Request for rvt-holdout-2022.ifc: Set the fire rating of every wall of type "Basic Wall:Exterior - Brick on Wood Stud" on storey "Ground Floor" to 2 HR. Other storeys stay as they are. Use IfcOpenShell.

First a look at what the model holds.

```python
import ifcopenshell
import ifcopenshell.util.element

model = ifcopenshell.open("rvt-holdout-2022.ifc")
print(model.schema)
storey = next(s for s in model.by_type("IfcBuildingStorey") if s.Name == "Ground Floor")
walls = [e for e in ifcopenshell.util.element.get_decomposition(storey) if e.is_a("IfcWall")]
seen = {}
for e in walls:
    element_type = ifcopenshell.util.element.get_type(e)
    key = (element_type.Name if element_type != e and element_type else None, ifcopenshell.util.element.get_pset(e, "Pset_WallCommon", "FireRating"))
    seen[key] = seen.get(key, 0) + 1
for (name, value), count in sorted(seen.items(), key=str):
    print(count, "x", name, "|", value)
```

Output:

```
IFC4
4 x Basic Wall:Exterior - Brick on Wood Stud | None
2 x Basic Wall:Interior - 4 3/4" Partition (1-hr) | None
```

```python
import ifcopenshell
import ifcopenshell.api.pset
import ifcopenshell.util.element

model = ifcopenshell.open("rvt-holdout-2022.ifc")

storey = next(s for s in model.by_type("IfcBuildingStorey") if s.Name == "Ground Floor")
walls = [e for e in ifcopenshell.util.element.get_decomposition(storey) if e.is_a("IfcWall")]

count = 0
for e in walls:
    element_type = ifcopenshell.util.element.get_type(e)
    if element_type in (None, e) or element_type.Name != "Basic Wall:Exterior - Brick on Wood Stud":
        continue
    # add_pset returns the element's existing set when there is one.
    pset = ifcopenshell.api.pset.add_pset(model, product=e, name="Pset_WallCommon")
    ifcopenshell.api.pset.edit_pset(model, pset=pset, properties={"FireRating": "2 HR"})
    count += 1

print(count, "walls updated")

model.write("rvt-holdout-2022-out.ifc")
```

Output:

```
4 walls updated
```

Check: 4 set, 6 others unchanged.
